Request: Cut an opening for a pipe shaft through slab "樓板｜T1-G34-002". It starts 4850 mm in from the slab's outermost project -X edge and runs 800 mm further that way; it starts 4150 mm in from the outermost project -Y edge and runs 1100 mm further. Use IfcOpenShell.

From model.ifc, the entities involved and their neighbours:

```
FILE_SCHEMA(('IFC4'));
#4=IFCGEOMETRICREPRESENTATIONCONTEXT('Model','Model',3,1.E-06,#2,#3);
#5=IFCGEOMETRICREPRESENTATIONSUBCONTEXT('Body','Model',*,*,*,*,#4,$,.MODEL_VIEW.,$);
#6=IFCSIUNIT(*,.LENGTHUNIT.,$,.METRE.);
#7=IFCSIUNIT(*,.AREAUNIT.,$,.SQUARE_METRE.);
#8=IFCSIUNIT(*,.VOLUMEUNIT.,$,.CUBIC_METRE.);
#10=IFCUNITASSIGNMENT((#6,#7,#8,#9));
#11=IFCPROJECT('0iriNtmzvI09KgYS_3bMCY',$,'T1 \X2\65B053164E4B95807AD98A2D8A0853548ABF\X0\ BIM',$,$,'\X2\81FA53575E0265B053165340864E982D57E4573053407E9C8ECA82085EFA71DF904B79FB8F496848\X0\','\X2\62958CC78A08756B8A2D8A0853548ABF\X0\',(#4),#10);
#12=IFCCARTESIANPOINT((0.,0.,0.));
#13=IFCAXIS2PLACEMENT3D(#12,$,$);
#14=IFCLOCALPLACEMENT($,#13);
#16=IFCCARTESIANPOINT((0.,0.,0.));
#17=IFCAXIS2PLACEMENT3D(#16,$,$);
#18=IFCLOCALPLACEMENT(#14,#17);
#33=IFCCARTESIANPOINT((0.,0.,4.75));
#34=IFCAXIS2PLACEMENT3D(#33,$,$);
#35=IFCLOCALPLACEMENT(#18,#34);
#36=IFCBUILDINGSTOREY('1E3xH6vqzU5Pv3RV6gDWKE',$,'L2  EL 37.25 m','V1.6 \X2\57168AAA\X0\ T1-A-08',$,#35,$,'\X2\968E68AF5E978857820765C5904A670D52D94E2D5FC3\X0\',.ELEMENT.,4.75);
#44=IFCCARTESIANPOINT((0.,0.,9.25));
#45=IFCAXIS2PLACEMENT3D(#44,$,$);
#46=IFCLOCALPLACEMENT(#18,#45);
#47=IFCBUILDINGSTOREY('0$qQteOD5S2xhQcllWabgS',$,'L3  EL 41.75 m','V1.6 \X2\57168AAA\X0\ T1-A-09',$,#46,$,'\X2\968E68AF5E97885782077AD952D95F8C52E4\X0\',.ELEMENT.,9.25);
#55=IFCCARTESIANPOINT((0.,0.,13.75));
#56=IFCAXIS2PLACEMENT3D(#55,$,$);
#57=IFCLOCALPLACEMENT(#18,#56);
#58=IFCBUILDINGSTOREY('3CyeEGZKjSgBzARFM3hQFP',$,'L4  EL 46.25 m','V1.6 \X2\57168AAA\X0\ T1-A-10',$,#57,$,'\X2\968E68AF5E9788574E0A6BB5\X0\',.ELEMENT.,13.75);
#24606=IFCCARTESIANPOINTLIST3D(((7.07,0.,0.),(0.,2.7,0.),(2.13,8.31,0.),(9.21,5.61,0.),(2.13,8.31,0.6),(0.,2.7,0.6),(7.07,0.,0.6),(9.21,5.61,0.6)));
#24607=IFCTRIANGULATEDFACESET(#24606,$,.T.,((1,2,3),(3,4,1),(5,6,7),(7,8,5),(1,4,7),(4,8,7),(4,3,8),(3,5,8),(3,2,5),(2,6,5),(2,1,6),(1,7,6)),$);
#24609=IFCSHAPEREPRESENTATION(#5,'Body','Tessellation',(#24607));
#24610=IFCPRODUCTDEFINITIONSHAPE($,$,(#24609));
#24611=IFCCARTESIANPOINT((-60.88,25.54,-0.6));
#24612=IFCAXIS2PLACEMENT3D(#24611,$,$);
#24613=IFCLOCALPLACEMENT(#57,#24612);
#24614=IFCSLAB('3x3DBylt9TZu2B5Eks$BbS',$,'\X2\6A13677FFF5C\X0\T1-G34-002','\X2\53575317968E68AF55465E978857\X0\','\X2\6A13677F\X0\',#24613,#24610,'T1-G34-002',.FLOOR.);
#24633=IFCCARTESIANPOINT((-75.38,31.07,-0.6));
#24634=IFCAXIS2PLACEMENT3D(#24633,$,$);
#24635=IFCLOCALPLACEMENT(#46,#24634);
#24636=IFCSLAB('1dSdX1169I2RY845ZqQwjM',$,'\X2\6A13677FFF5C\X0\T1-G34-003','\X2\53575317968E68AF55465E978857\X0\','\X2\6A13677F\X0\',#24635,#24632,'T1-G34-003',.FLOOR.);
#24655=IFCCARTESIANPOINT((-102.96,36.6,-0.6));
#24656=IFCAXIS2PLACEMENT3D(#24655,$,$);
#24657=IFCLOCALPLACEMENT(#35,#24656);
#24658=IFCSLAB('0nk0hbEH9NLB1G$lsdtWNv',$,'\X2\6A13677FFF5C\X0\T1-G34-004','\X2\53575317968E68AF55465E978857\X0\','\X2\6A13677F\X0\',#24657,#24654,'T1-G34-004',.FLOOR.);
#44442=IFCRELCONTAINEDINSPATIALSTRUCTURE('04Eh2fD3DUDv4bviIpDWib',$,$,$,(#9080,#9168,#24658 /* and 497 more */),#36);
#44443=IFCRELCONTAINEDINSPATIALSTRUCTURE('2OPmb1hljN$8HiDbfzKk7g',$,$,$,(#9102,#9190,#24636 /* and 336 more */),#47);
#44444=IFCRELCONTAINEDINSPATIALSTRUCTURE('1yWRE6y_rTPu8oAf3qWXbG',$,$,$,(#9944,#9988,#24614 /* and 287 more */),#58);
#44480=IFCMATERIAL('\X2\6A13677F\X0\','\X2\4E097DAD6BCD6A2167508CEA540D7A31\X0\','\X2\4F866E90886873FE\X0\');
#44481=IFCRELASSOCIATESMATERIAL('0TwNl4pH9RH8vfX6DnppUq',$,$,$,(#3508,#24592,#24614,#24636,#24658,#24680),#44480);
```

```python
import numpy as np
import ifcopenshell
import ifcopenshell.api.feature
import ifcopenshell.api.geometry
import ifcopenshell.api.root
import ifcopenshell.geom
import ifcopenshell.util.placement
import ifcopenshell.util.representation
import ifcopenshell.util.shape
import ifcopenshell.util.unit

model = ifcopenshell.open("model.ifc")
unit_scale = ifcopenshell.util.unit.calculate_unit_scale(model)
settings = ifcopenshell.geom.settings()


def volume(element):
    """Net volume in cubic metres, openings subtracted."""
    shape = ifcopenshell.geom.create_shape(settings, element)
    return ifcopenshell.util.shape.get_volume(shape.geometry)


slab = model.by_id(24614)
before = volume(slab)

# Extent in the slab's own axes, in metres. The edges named are its -X and -Y sides.
slab_shape = ifcopenshell.geom.create_shape(settings, slab)
vertices = ifcopenshell.util.shape.get_vertices(slab_shape.geometry)
x_min, y_min, bottom = vertices.min(axis=0)
top = vertices[:, 2].max()

opening = ifcopenshell.api.root.create_entity(model, ifc_class="IfcOpeningElement", name="Pipe shaft opening", predefined_type="OPENING")
context = ifcopenshell.util.representation.get_context(model, "Model", "Body", "MODEL_VIEW")
width, depth = 0.8, 1.1
outline = [(0.0, 0.0), (width, 0.0), (width, depth), (0.0, depth), (0.0, 0.0)]
# Overshoot both faces by 50 mm so the cut is clean.
shape = ifcopenshell.api.geometry.add_slab_representation(
    model, context=context, depth=top - bottom + 0.1, polyline=outline
)
ifcopenshell.api.geometry.assign_representation(model, product=opening, representation=shape)

matrix = ifcopenshell.util.placement.get_local_placement(slab.ObjectPlacement)
matrix[:, 3] = matrix @ np.append(np.array([x_min + 4.85, y_min + 4.15, bottom - 0.05]) / unit_scale, 1.0)
ifcopenshell.api.geometry.edit_object_placement(model, product=opening, matrix=matrix, is_si=False)
ifcopenshell.api.feature.add_feature(model, feature=opening, element=slab)

after = volume(slab)

print(f"slab volume {before:.3f} -> {after:.3f} m3")

model.write("model-out.ifc")
```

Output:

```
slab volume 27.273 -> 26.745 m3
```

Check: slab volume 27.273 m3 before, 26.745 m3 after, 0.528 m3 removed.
